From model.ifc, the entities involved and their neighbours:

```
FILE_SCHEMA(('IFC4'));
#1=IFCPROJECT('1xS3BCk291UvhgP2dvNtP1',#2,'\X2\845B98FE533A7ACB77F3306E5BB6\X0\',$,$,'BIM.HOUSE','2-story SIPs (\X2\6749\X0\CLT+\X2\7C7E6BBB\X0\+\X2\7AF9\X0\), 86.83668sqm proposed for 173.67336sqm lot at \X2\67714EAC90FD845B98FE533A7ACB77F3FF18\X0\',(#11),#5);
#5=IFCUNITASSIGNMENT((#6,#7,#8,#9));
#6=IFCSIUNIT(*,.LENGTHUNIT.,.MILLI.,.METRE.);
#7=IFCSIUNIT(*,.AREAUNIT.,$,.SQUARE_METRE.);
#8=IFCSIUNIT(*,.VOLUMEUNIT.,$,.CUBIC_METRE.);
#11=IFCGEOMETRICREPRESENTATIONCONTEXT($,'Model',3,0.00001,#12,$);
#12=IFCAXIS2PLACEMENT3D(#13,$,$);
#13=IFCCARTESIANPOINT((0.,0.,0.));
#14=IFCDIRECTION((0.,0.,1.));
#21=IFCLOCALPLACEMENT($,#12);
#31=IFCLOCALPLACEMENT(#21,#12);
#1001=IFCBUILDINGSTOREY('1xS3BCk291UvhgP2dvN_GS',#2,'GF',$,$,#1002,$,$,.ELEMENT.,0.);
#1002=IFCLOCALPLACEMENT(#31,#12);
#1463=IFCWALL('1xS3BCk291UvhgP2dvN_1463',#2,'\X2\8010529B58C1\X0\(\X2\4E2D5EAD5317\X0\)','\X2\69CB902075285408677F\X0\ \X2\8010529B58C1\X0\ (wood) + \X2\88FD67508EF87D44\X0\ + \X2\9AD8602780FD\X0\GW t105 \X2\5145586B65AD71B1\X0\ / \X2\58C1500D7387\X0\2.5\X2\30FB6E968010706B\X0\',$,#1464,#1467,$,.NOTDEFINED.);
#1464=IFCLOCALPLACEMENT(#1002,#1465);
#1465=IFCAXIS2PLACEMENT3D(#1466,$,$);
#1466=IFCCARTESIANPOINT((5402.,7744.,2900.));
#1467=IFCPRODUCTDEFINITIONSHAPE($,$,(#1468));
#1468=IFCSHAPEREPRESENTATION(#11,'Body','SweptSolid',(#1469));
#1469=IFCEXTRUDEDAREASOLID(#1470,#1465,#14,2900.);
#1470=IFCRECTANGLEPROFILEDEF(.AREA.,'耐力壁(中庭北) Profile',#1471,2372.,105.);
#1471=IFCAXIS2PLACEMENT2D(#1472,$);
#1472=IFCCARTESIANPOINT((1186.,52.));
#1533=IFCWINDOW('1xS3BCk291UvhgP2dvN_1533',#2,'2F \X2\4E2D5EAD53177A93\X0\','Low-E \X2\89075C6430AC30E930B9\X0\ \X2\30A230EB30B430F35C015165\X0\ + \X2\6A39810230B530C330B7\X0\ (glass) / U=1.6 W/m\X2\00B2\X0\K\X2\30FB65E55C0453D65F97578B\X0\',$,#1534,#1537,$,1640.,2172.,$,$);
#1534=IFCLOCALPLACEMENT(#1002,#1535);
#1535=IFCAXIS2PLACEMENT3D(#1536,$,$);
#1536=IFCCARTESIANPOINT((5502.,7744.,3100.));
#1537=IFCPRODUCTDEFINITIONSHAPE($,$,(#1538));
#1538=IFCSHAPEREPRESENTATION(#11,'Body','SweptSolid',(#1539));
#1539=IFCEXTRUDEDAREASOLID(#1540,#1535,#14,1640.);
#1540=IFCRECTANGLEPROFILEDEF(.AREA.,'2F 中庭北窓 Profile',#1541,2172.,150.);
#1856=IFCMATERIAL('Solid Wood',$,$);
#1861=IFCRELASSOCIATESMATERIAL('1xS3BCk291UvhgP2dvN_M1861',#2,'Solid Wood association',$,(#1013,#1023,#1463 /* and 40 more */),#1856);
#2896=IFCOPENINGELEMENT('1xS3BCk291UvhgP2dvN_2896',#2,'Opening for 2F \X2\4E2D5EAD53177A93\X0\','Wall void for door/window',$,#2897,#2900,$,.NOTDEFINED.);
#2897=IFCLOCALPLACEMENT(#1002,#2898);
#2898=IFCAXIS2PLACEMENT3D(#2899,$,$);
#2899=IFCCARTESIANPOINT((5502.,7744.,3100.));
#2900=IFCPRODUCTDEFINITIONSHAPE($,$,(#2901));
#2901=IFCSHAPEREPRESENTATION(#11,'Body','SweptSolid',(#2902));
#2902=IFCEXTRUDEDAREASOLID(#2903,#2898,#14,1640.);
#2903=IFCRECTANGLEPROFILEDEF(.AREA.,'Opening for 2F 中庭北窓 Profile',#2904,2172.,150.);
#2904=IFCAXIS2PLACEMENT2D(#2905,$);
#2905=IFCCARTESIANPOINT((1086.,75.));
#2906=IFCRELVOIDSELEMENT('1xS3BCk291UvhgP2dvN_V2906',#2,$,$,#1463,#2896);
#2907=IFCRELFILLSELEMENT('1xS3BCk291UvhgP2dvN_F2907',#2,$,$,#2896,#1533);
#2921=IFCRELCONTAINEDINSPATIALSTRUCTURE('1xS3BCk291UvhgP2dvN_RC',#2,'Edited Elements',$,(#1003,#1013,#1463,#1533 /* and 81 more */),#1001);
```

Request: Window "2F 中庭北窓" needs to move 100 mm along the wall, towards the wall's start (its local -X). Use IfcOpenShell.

```python
import ifcopenshell
import ifcopenshell.api.geometry
import ifcopenshell.util.placement

model = ifcopenshell.open("model.ifc")

window = model.by_id(1533)
opening = window.FillsVoids[0].RelatingOpeningElement
wall = opening.VoidsElements[0].RelatingBuildingElement

wall_matrix = ifcopenshell.util.placement.get_local_placement(wall.ObjectPlacement)
shift = wall_matrix[:3, 0] * -100.0
before = ifcopenshell.util.placement.get_local_placement(window.ObjectPlacement)[:3, 3].copy()

# The window is not placed relative to its opening, so move both.
for product in (opening, window):
    matrix = ifcopenshell.util.placement.get_local_placement(product.ObjectPlacement)
    matrix[:3, 3] += shift
    ifcopenshell.api.geometry.edit_object_placement(model, product=product, matrix=matrix, is_si=False)

after = ifcopenshell.util.placement.get_local_placement(window.ObjectPlacement)[:3, 3]
print("window moved by", (after - before).round(3) + 0.0)

model.write("model_rev.ifc")
```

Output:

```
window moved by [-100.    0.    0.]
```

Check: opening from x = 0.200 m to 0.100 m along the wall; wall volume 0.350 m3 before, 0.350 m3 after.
